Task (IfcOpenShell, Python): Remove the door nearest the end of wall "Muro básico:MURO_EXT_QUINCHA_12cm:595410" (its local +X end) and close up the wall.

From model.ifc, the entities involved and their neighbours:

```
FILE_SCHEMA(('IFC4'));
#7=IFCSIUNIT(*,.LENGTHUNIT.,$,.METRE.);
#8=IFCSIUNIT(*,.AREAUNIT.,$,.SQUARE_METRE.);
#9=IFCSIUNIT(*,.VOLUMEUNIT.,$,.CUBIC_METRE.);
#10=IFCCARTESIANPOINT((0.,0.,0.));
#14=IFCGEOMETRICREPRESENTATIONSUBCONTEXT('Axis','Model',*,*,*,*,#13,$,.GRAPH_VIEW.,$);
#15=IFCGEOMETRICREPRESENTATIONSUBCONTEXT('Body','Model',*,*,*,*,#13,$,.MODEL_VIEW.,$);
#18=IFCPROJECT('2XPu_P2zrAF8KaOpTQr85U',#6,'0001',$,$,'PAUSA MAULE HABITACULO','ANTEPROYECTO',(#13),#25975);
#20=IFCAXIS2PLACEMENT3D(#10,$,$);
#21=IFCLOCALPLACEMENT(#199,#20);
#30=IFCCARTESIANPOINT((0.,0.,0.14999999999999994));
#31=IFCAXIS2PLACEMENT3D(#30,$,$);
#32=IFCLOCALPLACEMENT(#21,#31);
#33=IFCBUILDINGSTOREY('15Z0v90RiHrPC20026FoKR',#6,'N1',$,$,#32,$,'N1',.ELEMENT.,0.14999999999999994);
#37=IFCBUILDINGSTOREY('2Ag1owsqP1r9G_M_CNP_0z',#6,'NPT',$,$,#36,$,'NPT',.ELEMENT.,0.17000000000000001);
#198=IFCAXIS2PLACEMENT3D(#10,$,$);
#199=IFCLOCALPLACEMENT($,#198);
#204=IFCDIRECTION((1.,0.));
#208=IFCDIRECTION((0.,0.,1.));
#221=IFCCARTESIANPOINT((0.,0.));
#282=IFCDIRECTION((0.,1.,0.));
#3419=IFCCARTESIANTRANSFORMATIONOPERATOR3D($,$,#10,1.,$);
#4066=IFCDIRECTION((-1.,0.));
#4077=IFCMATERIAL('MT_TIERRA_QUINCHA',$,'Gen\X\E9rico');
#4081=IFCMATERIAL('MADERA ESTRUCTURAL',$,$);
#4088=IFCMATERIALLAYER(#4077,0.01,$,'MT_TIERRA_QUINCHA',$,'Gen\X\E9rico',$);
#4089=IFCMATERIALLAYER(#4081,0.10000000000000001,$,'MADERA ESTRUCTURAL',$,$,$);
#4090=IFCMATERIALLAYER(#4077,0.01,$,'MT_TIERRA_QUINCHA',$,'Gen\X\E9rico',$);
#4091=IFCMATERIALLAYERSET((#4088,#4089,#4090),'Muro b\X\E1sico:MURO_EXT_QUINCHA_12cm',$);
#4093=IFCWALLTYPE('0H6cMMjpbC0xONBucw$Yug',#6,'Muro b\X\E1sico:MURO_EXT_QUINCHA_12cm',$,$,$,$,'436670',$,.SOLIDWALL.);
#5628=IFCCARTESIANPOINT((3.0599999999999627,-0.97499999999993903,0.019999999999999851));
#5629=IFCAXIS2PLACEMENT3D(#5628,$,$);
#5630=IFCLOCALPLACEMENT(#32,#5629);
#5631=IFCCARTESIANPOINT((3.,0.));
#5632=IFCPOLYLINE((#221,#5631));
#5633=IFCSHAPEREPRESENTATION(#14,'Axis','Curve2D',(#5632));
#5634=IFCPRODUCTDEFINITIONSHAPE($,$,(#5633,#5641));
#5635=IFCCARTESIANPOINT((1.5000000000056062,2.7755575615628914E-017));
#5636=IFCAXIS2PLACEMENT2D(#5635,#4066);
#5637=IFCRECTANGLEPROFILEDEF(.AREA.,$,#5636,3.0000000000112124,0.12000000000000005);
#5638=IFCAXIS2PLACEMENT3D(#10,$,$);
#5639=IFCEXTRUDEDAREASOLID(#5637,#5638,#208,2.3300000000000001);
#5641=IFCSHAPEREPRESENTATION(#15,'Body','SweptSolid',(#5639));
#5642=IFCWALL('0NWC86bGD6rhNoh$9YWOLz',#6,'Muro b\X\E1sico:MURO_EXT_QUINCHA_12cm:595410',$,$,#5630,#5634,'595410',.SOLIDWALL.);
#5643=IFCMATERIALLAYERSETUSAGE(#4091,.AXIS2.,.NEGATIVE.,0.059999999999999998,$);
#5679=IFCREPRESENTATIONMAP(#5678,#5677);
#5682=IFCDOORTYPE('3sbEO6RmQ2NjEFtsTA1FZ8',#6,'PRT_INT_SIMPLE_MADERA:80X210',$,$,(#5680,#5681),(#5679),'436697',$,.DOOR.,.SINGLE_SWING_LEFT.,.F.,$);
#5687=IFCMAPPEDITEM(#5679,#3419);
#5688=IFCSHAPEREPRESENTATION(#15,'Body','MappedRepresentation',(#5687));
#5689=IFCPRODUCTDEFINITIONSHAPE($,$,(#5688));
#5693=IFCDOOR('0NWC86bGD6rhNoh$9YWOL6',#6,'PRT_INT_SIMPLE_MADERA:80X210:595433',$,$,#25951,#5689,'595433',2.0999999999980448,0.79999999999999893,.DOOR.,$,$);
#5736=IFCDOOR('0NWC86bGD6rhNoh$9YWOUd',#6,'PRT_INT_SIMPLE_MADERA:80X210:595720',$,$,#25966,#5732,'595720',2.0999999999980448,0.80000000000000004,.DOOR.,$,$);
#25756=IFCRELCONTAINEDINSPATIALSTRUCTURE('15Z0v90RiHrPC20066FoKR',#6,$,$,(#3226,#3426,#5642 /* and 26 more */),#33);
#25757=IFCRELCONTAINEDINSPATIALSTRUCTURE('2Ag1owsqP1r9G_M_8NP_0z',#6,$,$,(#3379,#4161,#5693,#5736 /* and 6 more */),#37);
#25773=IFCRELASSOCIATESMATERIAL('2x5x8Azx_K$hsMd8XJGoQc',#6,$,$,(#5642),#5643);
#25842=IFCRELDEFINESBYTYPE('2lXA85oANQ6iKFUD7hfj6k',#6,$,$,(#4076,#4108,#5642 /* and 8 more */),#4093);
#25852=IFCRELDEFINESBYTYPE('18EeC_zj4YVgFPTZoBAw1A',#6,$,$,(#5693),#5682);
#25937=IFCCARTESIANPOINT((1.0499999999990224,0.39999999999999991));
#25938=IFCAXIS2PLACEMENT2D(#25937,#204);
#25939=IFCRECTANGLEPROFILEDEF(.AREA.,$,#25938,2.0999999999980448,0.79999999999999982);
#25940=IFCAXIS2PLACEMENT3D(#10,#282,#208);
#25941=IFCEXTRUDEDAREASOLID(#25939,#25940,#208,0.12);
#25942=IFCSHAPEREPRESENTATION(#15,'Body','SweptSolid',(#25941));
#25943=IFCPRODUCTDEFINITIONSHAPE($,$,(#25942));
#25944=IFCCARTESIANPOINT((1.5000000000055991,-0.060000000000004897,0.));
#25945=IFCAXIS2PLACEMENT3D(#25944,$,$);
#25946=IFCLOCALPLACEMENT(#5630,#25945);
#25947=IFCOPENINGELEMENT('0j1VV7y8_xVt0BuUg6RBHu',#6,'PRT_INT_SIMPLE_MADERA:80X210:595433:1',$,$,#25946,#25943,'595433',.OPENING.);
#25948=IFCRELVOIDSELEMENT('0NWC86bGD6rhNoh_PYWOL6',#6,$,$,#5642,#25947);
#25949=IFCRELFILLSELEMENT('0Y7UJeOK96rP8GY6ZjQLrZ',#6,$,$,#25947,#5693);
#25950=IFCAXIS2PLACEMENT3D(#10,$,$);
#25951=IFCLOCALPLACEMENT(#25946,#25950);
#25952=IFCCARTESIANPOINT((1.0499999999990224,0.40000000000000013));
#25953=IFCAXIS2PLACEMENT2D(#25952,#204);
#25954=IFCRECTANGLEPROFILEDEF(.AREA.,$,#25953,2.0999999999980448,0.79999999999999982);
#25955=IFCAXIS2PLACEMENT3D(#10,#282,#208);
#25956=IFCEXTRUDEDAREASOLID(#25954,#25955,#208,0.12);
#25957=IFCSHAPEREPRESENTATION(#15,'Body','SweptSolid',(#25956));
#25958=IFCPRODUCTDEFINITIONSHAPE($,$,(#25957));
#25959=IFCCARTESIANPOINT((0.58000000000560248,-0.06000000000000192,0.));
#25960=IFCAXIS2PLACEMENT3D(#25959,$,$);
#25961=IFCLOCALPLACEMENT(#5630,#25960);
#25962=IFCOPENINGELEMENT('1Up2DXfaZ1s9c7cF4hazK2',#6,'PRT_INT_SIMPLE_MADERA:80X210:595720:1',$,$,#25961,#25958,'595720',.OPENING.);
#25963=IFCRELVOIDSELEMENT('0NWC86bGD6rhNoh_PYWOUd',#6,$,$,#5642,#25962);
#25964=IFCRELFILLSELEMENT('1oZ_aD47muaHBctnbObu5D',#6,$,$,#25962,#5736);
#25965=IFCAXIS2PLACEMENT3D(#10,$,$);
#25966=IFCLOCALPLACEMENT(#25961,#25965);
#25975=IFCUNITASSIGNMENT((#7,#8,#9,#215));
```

```python
import ifcopenshell
import ifcopenshell.api.feature
import ifcopenshell.api.root
import ifcopenshell.geom
import ifcopenshell.util.shape

model = ifcopenshell.open("model.ifc")
settings = ifcopenshell.geom.settings()


def volume(element):
    """Net volume in cubic metres, openings subtracted."""
    shape = ifcopenshell.geom.create_shape(settings, element)
    return ifcopenshell.util.shape.get_volume(shape.geometry)


door = model.by_guid("0NWC86bGD6rhNoh$9YWOL6")
opening = door.FillsVoids[0].RelatingOpeningElement
wall = opening.VoidsElements[0].RelatingBuildingElement
before = volume(wall)

ifcopenshell.api.root.remove_product(model, product=door)
ifcopenshell.api.feature.remove_feature(model, feature=opening)

after = volume(wall)

print(f"wall volume {before:.3f} -> {after:.3f} m3")

model.write("model_v2.ifc")
```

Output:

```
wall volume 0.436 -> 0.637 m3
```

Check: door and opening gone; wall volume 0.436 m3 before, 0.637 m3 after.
